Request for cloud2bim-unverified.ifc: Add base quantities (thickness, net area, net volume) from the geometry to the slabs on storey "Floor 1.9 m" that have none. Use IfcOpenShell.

First a look at what the model holds.

```python
import ifcopenshell
import ifcopenshell.util.element
import ifcopenshell.util.unit

model = ifcopenshell.open("cloud2bim-unverified.ifc")
print(model.schema)
for unit_type in ("LENGTHUNIT", "AREAUNIT", "VOLUMEUNIT"):
    print(unit_type, ifcopenshell.util.unit.calculate_unit_scale(model, unit_type))
storey = next(s for s in model.by_type("IfcBuildingStorey") if s.Name == "Floor 1.9 m")
slabs = [e for e in ifcopenshell.util.element.get_decomposition(storey) if e.is_a("IfcSlab")]
for e in sorted(slabs, key=lambda e: e.id()):
    print(e.id(), e.is_a(), e.Name, list(ifcopenshell.util.element.get_psets(e, qtos_only=True)), sep=" | ")
```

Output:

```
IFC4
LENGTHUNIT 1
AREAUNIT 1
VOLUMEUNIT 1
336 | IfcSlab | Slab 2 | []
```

```python
import ifcopenshell
import ifcopenshell.api.pset
import ifcopenshell.geom
import ifcopenshell.util.element
import ifcopenshell.util.shape
import ifcopenshell.util.unit

model = ifcopenshell.open("cloud2bim-unverified.ifc")
unit_scale = ifcopenshell.util.unit.calculate_unit_scale(model)
area_scale = ifcopenshell.util.unit.calculate_unit_scale(model, "AREAUNIT")
volume_scale = ifcopenshell.util.unit.calculate_unit_scale(model, "VOLUMEUNIT")
settings = ifcopenshell.geom.settings()

storey = next(s for s in model.by_type("IfcBuildingStorey") if s.Name == "Floor 1.9 m")
slabs = [e for e in ifcopenshell.util.element.get_decomposition(storey) if e.is_a("IfcSlab")]

for e in sorted(slabs, key=lambda e: e.id()):
    if ifcopenshell.util.element.get_psets(e, qtos_only=True, should_inherit=False):
        continue
    # Geometry comes back in metres, in the element's own axes.
    shape = ifcopenshell.geom.create_shape(settings, e)
    values = {
        "Width": ifcopenshell.util.shape.get_z(shape.geometry) / unit_scale,
        "NetArea": ifcopenshell.util.shape.get_footprint_area(shape.geometry) / area_scale,
        "NetVolume": ifcopenshell.util.shape.get_volume(shape.geometry) / volume_scale,
    }
    qto = ifcopenshell.api.pset.add_qto(model, product=e, name="Qto_SlabBaseQuantities")
    ifcopenshell.api.pset.edit_qto(model, qto=qto, properties=values)
    print(e.id(), {k: round(v, 3) for k, v in values.items()})

model.write("cloud2bim-unverified_updated.ifc")
```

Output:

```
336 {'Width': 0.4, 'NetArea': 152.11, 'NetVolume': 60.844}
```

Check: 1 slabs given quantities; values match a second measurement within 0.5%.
